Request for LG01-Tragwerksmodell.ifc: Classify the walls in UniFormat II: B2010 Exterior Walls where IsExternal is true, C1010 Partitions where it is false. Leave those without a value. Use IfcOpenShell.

First a look at what the model holds.

```python
import ifcopenshell
import ifcopenshell.util.element

model = ifcopenshell.open("LG01-Tragwerksmodell.ifc")
print(model.schema)
print("classifications:", [c.Name for c in model.by_type("IfcClassification")])
values = [ifcopenshell.util.element.get_pset(e, "Pset_WallCommon", "IsExternal") for e in model.by_type("IfcWall")]
for value in (True, False, None):
    print("IsExternal", value, values.count(value))
```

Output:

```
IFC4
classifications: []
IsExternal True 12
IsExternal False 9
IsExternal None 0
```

```python
import ifcopenshell
import ifcopenshell.api.classification
import ifcopenshell.util.element

model = ifcopenshell.open("LG01-Tragwerksmodell.ifc")

system = ifcopenshell.api.classification.add_classification(model, classification="UniFormat II")

walls = model.by_type("IfcWall")
external = {e: ifcopenshell.util.element.get_pset(e, "Pset_WallCommon", "IsExternal") for e in walls}
for flag, code, name in ((True, "B2010", "Exterior Walls"), (False, "C1010", "Partitions")):
    products = [e for e in walls if external[e] is flag]
    ifcopenshell.api.classification.add_reference(
        model, products=products, classification=system, identification=code, name=name
    )
    print(code, len(products))

model.write("LG01-Tragwerksmodell_v2.ifc")
```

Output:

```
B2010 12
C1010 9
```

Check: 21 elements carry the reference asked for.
